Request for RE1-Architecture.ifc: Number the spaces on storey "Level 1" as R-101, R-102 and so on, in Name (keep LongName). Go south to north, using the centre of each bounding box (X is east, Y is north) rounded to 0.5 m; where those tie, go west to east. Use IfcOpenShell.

First a look at what the model holds.

```python
import ifcopenshell
import ifcopenshell.util.element
import ifcopenshell.util.placement

model = ifcopenshell.open("RE1-Architecture.ifc")
print(model.schema)
storey = next(s for s in model.by_type("IfcBuildingStorey") if s.Name == "Level 1")
spaces = [e for e in ifcopenshell.util.element.get_decomposition(storey) if e.is_a("IfcSpace")]
for e in sorted(spaces, key=lambda e: e.id()):
    origin = ifcopenshell.util.placement.get_local_placement(e.ObjectPlacement)[:3, 3]
    print(e.id(), e.Name, e.LongName, origin.round(2) + 0.0, sep=" | ")
```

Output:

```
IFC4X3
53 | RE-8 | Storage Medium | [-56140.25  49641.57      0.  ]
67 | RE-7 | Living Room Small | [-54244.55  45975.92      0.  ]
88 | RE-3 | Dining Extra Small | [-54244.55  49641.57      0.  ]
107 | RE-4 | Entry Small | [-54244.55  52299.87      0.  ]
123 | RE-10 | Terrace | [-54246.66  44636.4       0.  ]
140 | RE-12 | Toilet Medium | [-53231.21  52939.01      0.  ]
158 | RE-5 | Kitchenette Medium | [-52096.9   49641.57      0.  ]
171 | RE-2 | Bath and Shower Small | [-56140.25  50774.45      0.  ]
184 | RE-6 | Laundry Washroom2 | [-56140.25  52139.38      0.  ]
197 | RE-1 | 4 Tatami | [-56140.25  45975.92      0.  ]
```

```python
import ifcopenshell
import ifcopenshell.geom
import ifcopenshell.util.element
import ifcopenshell.util.shape

model = ifcopenshell.open("RE1-Architecture.ifc")
settings = ifcopenshell.geom.settings()
settings.set("use-world-coords", True)


def centre(element):
    shape = ifcopenshell.geom.create_shape(settings, element)
    return ifcopenshell.util.shape.get_bbox_centroid(shape.geometry)


storey = next(s for s in model.by_type("IfcBuildingStorey") if s.Name == "Level 1")
spaces = [e for e in ifcopenshell.util.element.get_decomposition(storey) if e.is_a("IfcSpace")]

# Insertion points can sit at a corner or the storey origin, so sort by the geometry (in metres).
centres = {e: centre(e) for e in spaces}
spaces.sort(key=lambda e: (round(centres[e][1] / 0.5), centres[e][0]))

for i, e in enumerate(spaces, start=1):
    number = f"R-1{i:02d}"
    e.Name = number
    print(e.id(), number)

model.write("RE1-Architecture-out.ifc")
```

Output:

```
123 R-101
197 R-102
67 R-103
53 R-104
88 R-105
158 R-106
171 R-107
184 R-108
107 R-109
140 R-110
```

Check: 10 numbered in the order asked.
